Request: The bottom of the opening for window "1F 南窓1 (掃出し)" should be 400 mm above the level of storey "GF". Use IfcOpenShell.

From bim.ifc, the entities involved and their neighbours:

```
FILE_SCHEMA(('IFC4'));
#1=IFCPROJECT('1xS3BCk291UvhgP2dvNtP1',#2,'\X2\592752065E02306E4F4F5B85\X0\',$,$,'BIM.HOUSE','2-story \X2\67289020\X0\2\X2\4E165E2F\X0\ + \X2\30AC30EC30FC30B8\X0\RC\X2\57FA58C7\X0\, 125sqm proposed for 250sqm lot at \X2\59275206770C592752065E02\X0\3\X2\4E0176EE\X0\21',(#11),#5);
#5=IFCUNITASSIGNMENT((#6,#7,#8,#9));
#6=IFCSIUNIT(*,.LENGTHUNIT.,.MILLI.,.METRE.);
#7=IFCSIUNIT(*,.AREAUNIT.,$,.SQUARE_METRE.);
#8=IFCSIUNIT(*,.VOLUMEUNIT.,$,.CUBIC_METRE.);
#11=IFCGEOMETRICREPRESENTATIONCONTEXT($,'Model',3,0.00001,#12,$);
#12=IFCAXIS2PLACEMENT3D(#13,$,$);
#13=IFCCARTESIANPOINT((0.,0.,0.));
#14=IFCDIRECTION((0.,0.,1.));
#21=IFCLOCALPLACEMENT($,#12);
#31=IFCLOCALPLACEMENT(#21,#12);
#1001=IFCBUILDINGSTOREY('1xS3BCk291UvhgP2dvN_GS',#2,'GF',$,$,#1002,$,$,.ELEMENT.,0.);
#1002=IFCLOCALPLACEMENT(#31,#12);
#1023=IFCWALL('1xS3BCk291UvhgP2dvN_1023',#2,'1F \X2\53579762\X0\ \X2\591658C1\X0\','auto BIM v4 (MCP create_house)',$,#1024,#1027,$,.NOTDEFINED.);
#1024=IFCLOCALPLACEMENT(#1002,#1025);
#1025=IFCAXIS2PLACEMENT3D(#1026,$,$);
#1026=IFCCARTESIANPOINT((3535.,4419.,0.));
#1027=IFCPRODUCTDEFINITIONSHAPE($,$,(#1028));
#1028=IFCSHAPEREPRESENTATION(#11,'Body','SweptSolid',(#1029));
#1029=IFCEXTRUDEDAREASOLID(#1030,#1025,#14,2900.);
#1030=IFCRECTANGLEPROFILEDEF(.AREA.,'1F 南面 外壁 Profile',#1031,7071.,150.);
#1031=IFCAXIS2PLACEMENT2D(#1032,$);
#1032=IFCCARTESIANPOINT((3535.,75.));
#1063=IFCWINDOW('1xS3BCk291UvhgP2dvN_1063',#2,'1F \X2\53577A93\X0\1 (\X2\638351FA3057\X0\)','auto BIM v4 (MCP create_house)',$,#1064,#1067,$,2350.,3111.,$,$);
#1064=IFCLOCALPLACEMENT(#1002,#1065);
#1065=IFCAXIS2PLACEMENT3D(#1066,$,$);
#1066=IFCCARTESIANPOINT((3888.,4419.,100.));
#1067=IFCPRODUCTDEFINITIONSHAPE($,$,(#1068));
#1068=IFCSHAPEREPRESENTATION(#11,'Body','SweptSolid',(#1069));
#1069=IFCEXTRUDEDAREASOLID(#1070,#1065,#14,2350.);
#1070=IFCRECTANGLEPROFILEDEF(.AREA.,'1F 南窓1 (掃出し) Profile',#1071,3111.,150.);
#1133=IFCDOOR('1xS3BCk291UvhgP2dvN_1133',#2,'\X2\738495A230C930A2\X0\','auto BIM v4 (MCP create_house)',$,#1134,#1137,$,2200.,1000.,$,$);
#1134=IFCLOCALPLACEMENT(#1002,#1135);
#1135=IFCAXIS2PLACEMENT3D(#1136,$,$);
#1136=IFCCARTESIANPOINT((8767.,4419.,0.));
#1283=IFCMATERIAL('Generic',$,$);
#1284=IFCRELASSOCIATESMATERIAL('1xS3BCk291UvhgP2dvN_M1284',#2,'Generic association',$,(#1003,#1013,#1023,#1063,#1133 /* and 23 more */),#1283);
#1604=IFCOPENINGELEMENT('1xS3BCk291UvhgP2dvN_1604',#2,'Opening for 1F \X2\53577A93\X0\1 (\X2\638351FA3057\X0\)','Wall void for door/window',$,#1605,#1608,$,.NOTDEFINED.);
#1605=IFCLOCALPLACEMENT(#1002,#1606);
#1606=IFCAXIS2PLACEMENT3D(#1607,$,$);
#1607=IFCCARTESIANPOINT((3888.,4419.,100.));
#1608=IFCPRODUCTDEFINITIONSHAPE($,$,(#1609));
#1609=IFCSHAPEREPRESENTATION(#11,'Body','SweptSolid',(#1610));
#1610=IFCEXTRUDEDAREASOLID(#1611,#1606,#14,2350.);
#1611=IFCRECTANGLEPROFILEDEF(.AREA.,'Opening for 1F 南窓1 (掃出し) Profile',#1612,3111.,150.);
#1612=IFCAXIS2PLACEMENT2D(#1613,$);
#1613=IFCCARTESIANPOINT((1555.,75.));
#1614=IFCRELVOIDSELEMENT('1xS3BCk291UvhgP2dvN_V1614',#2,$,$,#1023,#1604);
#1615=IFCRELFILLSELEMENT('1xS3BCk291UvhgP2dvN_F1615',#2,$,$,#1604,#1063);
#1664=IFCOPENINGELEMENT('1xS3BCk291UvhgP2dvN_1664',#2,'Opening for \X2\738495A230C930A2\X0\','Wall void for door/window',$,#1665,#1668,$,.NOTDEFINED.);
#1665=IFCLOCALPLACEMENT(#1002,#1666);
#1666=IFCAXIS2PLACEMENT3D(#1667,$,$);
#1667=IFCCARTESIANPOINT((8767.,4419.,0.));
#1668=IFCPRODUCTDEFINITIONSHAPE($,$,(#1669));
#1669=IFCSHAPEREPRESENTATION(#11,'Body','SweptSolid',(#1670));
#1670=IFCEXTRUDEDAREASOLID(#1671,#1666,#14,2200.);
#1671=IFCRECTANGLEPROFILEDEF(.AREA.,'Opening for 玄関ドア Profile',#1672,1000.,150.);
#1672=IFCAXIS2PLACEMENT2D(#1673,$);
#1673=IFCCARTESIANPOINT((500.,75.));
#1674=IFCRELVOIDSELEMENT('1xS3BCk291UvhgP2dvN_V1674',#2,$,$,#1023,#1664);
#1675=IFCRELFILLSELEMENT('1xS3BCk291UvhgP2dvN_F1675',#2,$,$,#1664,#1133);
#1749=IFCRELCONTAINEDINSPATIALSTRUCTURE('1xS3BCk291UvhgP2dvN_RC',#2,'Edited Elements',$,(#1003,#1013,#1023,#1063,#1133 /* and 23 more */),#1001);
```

```python
import numpy as np
import ifcopenshell
import ifcopenshell.api.geometry
import ifcopenshell.geom
import ifcopenshell.util.element
import ifcopenshell.util.placement
import ifcopenshell.util.shape
import ifcopenshell.util.unit

model = ifcopenshell.open("bim.ifc")
unit_scale = ifcopenshell.util.unit.calculate_unit_scale(model)

window = model.by_guid("1xS3BCk291UvhgP2dvN_1063")
opening = window.FillsVoids[0].RelatingOpeningElement
storey = ifcopenshell.util.element.get_container(window, ifc_class="IfcBuildingStorey")
level = ifcopenshell.util.placement.get_local_placement(storey.ObjectPlacement)[2, 3]

# The opening's origin need not be at the sill, so measure its lowest point.
shape = ifcopenshell.geom.create_shape(ifcopenshell.geom.settings(), opening)
bottom = ifcopenshell.util.shape.get_shape_bottom_elevation(shape, shape.geometry) / unit_scale
dz = level + 400.0 - bottom

shift = np.array([0.0, 0.0, dz])
# The window is not placed relative to its opening, so move both.
for product in (opening, window):
    matrix = ifcopenshell.util.placement.get_local_placement(product.ObjectPlacement)
    matrix[:3, 3] += shift
    ifcopenshell.api.geometry.edit_object_placement(model, product=product, matrix=matrix, is_si=False)

print(f"moved by {dz * unit_scale:+.3f} m")

model.write("bim-out.ifc")
```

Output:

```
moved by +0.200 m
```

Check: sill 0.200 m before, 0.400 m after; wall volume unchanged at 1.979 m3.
